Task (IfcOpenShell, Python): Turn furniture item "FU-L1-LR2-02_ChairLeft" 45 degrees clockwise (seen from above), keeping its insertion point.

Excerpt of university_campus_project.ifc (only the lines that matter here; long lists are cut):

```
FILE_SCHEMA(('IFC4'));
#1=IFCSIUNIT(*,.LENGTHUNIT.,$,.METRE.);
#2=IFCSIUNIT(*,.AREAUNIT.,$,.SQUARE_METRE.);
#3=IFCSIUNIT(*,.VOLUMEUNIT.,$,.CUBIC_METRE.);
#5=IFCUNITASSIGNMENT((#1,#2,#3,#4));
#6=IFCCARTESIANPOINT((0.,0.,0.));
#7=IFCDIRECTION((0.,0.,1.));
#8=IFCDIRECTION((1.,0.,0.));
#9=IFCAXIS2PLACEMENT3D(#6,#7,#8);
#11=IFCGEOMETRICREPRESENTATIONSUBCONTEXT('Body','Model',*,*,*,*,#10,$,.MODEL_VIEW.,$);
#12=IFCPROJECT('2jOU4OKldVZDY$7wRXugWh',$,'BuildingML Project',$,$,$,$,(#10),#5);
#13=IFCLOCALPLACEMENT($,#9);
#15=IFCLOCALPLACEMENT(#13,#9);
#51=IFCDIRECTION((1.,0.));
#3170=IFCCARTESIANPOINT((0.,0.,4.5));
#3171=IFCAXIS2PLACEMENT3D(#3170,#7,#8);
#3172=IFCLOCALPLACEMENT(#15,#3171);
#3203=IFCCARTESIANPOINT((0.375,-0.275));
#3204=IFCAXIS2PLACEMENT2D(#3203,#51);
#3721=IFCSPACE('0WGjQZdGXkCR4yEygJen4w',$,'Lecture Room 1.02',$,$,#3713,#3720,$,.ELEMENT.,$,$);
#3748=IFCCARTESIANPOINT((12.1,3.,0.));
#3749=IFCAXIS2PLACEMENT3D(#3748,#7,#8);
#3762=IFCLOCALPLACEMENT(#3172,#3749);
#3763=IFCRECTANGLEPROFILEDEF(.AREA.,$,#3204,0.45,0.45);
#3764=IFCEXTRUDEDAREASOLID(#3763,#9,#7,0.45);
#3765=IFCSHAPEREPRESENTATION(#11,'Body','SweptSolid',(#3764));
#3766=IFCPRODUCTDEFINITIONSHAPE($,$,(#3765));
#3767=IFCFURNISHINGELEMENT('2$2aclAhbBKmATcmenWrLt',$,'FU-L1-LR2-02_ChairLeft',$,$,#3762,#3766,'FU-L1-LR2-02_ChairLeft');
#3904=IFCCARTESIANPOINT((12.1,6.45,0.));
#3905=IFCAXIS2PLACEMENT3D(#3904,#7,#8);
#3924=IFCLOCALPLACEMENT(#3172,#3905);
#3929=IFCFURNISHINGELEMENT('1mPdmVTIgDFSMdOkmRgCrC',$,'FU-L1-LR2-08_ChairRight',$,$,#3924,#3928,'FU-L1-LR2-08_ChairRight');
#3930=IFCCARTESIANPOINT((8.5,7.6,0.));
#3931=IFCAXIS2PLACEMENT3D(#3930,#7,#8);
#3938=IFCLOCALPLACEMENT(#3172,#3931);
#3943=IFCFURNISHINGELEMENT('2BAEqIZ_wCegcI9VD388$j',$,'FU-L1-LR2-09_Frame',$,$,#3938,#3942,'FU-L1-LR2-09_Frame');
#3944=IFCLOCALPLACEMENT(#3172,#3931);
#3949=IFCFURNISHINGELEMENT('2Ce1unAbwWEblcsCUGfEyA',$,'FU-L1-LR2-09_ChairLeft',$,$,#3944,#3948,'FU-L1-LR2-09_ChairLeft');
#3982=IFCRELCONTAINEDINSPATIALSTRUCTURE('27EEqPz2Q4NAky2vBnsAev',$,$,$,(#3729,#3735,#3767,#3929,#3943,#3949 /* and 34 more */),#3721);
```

```python
import ifcopenshell
import ifcopenshell.api.geometry
import ifcopenshell.util.placement

model = ifcopenshell.open("university_campus_project.ifc")

item = model.by_guid("2$2aclAhbBKmATcmenWrLt")
matrix = ifcopenshell.util.placement.get_local_placement(item.ObjectPlacement)
matrix = matrix @ ifcopenshell.util.placement.rotation(-45, "Z")
ifcopenshell.api.geometry.edit_object_placement(model, product=item, matrix=matrix, is_si=False)

print(ifcopenshell.util.placement.get_local_placement(item.ObjectPlacement).round(3) + 0.0)

model.write("university_campus_project_v2.ifc")
```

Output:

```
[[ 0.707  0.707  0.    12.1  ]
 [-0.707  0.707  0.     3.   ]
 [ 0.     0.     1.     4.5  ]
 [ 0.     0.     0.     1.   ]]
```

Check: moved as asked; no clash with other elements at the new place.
